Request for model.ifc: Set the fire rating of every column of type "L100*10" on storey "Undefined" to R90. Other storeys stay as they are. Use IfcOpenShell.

First a look at what the model holds.

```python
import ifcopenshell
import ifcopenshell.util.element

model = ifcopenshell.open("model.ifc")
print(model.schema)
storey = next(s for s in model.by_type("IfcBuildingStorey") if s.Name == "Undefined")
columns = [e for e in ifcopenshell.util.element.get_decomposition(storey) if e.is_a("IfcColumn")]
seen = {}
for e in columns:
    element_type = ifcopenshell.util.element.get_type(e)
    key = (element_type.Name if element_type != e and element_type else None, ifcopenshell.util.element.get_pset(e, "Pset_ColumnCommon", "FireRating"))
    seen[key] = seen.get(key, 0) + 1
for (name, value), count in sorted(seen.items(), key=str):
    print(count, "x", name, "|", value)
```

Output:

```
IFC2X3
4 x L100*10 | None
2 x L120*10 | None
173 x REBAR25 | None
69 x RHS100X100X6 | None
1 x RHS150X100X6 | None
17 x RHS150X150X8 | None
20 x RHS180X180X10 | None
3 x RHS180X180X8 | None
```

```python
import ifcopenshell
import ifcopenshell.api.pset
import ifcopenshell.util.element

model = ifcopenshell.open("model.ifc")

storey = next(s for s in model.by_type("IfcBuildingStorey") if s.Name == "Undefined")
columns = [e for e in ifcopenshell.util.element.get_decomposition(storey) if e.is_a("IfcColumn")]

count = 0
for e in columns:
    element_type = ifcopenshell.util.element.get_type(e)
    if element_type in (None, e) or element_type.Name != "L100*10":
        continue
    found = ifcopenshell.util.element.get_pset(e, "Pset_ColumnCommon", should_inherit=False)
    if found:
        pset = model.by_id(found["id"])
        if len(ifcopenshell.util.element.get_elements_by_pset(pset)) > 1:
            pset = ifcopenshell.api.pset.unshare_pset(model, products=[e], pset=pset)[0]
    else:
        pset = ifcopenshell.api.pset.add_pset(model, product=e, name="Pset_ColumnCommon")
    ifcopenshell.api.pset.edit_pset(model, pset=pset, properties={"FireRating": "R90"})
    count += 1

print(count, "columns updated")

model.write("model-out.ifc")
```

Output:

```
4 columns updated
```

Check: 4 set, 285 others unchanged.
